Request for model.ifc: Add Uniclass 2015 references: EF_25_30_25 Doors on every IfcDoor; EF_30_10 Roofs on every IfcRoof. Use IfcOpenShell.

First a look at what the model holds.

```python
import ifcopenshell

model = ifcopenshell.open("model.ifc")
print(model.schema)
print("classifications:", [c.Name for c in model.by_type("IfcClassification")])
for ifc_class in ("IfcDoor", "IfcRoof", "IfcStair", "IfcWall", "IfcWindow"):
    print(ifc_class, len(model.by_type(ifc_class)))
```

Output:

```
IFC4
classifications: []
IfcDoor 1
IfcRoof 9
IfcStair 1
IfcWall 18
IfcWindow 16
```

```python
import ifcopenshell
import ifcopenshell.api.classification

model = ifcopenshell.open("model.ifc")

system = ifcopenshell.api.classification.add_classification(model, classification="Uniclass 2015")

codes = {
    "IfcDoor": ("EF_25_30_25", "Doors"),
    "IfcRoof": ("EF_30_10", "Roofs"),
}
for ifc_class, (code, name) in codes.items():
    products = model.by_type(ifc_class)
    ifcopenshell.api.classification.add_reference(
        model, products=products, classification=system, identification=code, name=name
    )
    print(code, len(products))

model.write("model_rev.ifc")
```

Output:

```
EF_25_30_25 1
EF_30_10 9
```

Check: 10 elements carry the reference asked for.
